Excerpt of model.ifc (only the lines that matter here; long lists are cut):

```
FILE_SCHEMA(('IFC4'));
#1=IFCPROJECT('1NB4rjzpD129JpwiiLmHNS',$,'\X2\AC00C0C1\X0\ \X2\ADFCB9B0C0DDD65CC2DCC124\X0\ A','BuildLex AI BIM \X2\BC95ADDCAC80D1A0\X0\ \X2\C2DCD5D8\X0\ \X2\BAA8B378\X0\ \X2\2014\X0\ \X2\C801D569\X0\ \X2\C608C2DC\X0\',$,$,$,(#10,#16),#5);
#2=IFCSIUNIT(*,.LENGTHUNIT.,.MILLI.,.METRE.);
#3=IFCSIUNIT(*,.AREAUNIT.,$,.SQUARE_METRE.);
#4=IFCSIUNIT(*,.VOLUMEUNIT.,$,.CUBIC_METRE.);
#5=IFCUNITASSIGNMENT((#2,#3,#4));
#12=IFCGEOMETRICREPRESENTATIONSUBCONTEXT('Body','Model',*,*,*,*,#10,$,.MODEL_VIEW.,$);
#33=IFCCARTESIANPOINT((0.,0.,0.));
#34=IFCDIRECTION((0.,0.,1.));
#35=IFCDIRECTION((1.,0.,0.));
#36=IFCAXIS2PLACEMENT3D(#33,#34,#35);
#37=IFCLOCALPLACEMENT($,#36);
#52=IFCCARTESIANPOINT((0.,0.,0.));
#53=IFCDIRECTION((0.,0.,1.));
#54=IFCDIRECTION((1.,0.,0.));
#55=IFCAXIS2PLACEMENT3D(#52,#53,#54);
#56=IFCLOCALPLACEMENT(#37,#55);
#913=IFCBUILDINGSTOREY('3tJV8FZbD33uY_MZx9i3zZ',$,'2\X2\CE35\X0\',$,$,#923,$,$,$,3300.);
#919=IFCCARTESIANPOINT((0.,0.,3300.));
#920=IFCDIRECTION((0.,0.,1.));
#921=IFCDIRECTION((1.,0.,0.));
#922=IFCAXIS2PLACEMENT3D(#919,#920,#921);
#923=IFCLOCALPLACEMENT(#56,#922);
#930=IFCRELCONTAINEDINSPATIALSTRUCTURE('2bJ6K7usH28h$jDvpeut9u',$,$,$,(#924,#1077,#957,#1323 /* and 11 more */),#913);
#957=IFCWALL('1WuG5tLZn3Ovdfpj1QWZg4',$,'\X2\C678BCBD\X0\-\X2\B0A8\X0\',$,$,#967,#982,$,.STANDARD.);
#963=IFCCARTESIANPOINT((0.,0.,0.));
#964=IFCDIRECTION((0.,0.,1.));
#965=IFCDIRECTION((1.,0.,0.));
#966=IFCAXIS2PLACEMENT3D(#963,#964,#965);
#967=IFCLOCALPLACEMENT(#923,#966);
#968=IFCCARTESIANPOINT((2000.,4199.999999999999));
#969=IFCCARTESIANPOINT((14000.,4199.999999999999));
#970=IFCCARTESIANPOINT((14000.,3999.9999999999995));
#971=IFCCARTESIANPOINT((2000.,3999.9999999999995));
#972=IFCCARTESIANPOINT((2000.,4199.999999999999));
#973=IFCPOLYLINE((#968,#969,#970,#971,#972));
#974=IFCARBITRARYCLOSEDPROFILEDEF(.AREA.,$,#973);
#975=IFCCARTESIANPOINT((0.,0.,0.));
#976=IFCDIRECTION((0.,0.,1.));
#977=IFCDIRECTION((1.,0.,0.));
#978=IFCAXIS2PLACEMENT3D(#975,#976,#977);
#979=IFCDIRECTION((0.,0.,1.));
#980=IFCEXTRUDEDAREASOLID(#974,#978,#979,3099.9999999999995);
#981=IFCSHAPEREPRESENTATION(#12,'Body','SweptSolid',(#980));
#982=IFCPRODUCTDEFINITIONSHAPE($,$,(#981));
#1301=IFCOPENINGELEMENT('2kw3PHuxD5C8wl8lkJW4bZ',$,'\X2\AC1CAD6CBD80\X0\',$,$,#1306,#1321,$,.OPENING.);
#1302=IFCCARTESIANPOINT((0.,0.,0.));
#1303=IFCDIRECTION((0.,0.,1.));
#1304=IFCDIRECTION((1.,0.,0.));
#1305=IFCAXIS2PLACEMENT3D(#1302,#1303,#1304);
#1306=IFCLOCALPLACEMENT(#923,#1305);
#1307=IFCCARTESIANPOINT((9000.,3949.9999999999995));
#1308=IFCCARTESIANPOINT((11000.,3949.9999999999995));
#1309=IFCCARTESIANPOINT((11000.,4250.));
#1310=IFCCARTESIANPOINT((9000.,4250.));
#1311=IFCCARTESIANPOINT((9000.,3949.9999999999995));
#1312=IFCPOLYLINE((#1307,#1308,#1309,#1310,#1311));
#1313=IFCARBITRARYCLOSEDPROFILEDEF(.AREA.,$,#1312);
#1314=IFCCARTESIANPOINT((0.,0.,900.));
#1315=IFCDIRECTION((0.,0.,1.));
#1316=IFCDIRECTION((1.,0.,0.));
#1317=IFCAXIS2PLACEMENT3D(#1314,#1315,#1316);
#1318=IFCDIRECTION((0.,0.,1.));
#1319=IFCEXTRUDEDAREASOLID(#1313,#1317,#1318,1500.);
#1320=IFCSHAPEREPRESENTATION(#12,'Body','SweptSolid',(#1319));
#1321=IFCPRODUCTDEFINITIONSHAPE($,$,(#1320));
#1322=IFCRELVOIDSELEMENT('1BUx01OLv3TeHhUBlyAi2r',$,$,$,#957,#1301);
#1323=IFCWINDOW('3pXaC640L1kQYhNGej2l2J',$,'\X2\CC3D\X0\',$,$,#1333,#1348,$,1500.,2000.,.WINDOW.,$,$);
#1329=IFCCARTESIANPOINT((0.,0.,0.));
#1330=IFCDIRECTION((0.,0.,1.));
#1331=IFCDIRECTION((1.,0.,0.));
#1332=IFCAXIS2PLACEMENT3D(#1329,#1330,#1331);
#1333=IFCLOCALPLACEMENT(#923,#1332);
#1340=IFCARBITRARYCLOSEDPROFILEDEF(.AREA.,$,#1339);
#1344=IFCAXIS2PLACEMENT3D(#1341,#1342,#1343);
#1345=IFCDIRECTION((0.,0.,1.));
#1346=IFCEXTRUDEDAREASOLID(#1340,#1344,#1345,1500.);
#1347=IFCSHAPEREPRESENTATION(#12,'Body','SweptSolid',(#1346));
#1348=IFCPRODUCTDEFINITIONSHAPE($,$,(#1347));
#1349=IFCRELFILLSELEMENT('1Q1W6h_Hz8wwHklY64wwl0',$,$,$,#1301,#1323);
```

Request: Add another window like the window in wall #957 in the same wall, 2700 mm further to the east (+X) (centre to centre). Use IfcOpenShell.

```python
import ifcopenshell
import ifcopenshell.api.feature
import ifcopenshell.api.geometry
import ifcopenshell.api.root
import ifcopenshell.geom
import ifcopenshell.util.element
import ifcopenshell.util.placement
import ifcopenshell.util.shape
import ifcopenshell.util.unit

model = ifcopenshell.open("model.ifc")
unit_scale = ifcopenshell.util.unit.calculate_unit_scale(model)
settings = ifcopenshell.geom.settings()


def volume(element):
    """Net volume in cubic metres, openings subtracted."""
    shape = ifcopenshell.geom.create_shape(settings, element)
    return ifcopenshell.util.shape.get_volume(shape.geometry)


window = model.by_id(1323)
opening = window.FillsVoids[0].RelatingOpeningElement
wall = opening.VoidsElements[0].RelatingBuildingElement
before = volume(wall)
shift = ifcopenshell.util.placement.get_local_placement(wall.ObjectPlacement)[:3, 0] * 2.7 / unit_scale

# copy_class copies the void relationship, type, container and properties, but no geometry.
new_opening = ifcopenshell.api.root.copy_class(model, product=opening)
new_opening.Representation = ifcopenshell.util.element.copy_deep(
    model, opening.Representation, exclude=["IfcGeometricRepresentationContext", "IfcRepresentationMap"]
)
new_window = ifcopenshell.api.root.copy_class(model, product=window)
new_window.Representation = ifcopenshell.util.element.copy_deep(
    model, window.Representation, exclude=["IfcGeometricRepresentationContext", "IfcRepresentationMap"]
)
ifcopenshell.api.feature.add_filling(model, opening=new_opening, element=new_window)

for old, new in ((opening, new_opening), (window, new_window)):
    matrix = ifcopenshell.util.placement.get_local_placement(old.ObjectPlacement)
    matrix[:3, 3] += shift
    ifcopenshell.api.geometry.edit_object_placement(model, product=new, matrix=matrix, is_si=False)

after = volume(wall)

print(f"wall volume {before:.3f} -> {after:.3f} m3")

model.write("model_v2.ifc")
```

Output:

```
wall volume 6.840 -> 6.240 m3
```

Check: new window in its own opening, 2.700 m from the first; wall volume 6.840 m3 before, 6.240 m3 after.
